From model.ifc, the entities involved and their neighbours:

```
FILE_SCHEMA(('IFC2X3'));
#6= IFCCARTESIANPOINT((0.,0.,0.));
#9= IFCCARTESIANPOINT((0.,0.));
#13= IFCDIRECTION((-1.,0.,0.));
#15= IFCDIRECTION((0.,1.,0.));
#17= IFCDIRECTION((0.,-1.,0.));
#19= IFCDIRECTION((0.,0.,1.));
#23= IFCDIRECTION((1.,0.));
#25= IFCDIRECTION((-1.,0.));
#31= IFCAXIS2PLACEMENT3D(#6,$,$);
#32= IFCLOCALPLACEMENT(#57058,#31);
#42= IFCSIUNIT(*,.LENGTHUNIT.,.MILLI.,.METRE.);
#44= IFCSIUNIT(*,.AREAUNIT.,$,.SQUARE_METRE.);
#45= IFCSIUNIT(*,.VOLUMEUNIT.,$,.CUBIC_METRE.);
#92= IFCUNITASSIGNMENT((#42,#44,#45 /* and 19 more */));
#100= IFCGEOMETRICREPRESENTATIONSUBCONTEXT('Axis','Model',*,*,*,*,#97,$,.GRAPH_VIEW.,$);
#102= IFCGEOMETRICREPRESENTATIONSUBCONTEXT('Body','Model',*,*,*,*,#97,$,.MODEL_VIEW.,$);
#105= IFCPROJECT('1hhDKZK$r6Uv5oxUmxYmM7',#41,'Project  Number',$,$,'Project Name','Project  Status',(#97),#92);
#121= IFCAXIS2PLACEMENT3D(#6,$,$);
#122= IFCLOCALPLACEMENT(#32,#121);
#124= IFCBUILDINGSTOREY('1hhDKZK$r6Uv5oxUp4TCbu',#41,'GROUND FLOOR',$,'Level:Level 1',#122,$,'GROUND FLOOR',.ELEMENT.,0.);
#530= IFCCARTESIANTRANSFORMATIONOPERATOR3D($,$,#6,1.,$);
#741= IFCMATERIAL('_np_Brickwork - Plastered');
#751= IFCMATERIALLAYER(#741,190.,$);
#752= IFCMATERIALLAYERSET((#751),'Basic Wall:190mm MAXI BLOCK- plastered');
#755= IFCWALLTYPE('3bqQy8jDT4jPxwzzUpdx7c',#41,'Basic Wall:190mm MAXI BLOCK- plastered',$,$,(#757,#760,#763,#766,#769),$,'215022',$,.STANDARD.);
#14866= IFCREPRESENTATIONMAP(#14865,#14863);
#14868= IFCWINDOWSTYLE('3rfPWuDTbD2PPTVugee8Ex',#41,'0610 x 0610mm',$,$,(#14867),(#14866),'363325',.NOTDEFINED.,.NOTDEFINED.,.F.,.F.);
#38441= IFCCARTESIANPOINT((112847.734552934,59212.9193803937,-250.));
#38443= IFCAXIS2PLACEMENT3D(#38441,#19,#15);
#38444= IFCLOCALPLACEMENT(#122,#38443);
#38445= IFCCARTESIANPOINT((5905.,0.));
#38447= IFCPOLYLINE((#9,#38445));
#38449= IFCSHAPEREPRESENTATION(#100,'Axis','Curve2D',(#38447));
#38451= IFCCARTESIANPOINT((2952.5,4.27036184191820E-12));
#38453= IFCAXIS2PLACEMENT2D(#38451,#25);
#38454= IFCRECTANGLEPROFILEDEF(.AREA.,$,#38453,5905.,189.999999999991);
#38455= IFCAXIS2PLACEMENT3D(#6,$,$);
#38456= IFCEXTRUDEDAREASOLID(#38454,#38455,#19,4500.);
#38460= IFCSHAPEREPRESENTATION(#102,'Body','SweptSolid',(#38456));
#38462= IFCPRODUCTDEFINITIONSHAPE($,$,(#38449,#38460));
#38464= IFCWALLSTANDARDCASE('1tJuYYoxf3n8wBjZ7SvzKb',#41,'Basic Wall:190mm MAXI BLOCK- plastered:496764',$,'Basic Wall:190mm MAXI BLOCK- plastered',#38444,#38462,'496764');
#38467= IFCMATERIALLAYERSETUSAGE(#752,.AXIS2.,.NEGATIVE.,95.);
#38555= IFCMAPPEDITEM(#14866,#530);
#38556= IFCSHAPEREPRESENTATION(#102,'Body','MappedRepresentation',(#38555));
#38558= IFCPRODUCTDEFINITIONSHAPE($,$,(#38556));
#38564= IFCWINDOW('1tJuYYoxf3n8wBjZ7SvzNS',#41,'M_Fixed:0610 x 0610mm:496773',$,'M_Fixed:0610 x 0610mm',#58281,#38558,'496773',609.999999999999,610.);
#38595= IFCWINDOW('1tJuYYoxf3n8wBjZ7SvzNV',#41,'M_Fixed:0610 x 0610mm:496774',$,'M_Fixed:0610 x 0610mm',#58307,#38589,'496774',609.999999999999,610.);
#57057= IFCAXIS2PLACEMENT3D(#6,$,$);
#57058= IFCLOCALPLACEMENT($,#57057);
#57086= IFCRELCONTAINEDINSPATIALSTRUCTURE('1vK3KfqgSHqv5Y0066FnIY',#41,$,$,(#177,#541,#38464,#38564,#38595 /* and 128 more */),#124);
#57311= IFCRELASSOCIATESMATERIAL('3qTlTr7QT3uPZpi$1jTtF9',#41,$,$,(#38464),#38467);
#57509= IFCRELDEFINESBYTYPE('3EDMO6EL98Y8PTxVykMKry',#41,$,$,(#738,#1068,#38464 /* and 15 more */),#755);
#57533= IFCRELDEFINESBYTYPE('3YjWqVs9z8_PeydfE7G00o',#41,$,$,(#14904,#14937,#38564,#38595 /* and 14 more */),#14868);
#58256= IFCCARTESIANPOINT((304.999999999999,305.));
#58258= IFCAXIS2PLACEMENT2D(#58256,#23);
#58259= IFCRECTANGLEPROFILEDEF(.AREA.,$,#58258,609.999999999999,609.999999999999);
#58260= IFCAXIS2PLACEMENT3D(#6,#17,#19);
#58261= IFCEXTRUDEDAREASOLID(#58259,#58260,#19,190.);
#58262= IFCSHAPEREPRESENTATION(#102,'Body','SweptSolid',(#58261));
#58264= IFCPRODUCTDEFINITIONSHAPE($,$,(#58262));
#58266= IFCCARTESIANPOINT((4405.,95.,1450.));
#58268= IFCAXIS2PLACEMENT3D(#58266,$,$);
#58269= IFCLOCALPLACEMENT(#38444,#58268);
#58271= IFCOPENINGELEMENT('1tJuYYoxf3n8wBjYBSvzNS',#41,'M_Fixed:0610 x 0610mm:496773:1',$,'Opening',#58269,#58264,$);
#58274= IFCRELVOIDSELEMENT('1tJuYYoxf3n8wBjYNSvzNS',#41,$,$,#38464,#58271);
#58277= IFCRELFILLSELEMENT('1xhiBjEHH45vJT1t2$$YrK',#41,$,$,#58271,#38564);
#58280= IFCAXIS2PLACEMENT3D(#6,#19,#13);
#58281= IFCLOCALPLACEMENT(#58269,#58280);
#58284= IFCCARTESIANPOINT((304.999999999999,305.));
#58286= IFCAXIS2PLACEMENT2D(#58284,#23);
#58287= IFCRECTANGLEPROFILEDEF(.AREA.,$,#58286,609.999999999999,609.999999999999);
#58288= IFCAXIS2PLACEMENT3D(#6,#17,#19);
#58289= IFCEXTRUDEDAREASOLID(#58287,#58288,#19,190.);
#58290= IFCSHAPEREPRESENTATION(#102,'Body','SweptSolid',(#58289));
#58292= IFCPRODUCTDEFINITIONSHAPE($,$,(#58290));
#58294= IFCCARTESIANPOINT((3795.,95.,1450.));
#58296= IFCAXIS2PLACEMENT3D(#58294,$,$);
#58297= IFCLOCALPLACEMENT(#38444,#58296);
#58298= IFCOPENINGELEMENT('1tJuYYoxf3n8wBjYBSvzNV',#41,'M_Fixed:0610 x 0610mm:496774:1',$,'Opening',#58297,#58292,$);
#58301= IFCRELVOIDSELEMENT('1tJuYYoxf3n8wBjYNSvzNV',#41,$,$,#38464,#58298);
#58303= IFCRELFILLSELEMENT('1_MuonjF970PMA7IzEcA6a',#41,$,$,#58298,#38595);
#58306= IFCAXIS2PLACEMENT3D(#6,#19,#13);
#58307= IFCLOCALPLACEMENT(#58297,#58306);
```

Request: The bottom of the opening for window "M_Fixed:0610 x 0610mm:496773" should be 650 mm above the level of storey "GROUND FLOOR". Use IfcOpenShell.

```python
import numpy as np
import ifcopenshell
import ifcopenshell.api.geometry
import ifcopenshell.geom
import ifcopenshell.util.element
import ifcopenshell.util.placement
import ifcopenshell.util.shape
import ifcopenshell.util.unit

model = ifcopenshell.open("model.ifc")
unit_scale = ifcopenshell.util.unit.calculate_unit_scale(model)

window = model.by_guid("1tJuYYoxf3n8wBjZ7SvzNS")
opening = window.FillsVoids[0].RelatingOpeningElement
storey = ifcopenshell.util.element.get_container(window, ifc_class="IfcBuildingStorey")
level = ifcopenshell.util.placement.get_local_placement(storey.ObjectPlacement)[2, 3]

# The opening's origin need not be at the sill, so measure its lowest point.
shape = ifcopenshell.geom.create_shape(ifcopenshell.geom.settings(), opening)
bottom = ifcopenshell.util.shape.get_shape_bottom_elevation(shape, shape.geometry) / unit_scale
dz = level + 0.65 / unit_scale - bottom

shift = np.array([0.0, 0.0, dz])
# The window is placed relative to its opening, so it follows when the opening moves.
matrix = ifcopenshell.util.placement.get_local_placement(opening.ObjectPlacement)
matrix[:3, 3] += shift
ifcopenshell.api.geometry.edit_object_placement(
    model, product=opening, matrix=matrix, is_si=False, should_transform_children=True
)

print(f"moved by {dz * unit_scale:+.3f} m")

model.write("model-out.ifc")
```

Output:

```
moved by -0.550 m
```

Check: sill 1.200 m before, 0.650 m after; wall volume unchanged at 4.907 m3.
